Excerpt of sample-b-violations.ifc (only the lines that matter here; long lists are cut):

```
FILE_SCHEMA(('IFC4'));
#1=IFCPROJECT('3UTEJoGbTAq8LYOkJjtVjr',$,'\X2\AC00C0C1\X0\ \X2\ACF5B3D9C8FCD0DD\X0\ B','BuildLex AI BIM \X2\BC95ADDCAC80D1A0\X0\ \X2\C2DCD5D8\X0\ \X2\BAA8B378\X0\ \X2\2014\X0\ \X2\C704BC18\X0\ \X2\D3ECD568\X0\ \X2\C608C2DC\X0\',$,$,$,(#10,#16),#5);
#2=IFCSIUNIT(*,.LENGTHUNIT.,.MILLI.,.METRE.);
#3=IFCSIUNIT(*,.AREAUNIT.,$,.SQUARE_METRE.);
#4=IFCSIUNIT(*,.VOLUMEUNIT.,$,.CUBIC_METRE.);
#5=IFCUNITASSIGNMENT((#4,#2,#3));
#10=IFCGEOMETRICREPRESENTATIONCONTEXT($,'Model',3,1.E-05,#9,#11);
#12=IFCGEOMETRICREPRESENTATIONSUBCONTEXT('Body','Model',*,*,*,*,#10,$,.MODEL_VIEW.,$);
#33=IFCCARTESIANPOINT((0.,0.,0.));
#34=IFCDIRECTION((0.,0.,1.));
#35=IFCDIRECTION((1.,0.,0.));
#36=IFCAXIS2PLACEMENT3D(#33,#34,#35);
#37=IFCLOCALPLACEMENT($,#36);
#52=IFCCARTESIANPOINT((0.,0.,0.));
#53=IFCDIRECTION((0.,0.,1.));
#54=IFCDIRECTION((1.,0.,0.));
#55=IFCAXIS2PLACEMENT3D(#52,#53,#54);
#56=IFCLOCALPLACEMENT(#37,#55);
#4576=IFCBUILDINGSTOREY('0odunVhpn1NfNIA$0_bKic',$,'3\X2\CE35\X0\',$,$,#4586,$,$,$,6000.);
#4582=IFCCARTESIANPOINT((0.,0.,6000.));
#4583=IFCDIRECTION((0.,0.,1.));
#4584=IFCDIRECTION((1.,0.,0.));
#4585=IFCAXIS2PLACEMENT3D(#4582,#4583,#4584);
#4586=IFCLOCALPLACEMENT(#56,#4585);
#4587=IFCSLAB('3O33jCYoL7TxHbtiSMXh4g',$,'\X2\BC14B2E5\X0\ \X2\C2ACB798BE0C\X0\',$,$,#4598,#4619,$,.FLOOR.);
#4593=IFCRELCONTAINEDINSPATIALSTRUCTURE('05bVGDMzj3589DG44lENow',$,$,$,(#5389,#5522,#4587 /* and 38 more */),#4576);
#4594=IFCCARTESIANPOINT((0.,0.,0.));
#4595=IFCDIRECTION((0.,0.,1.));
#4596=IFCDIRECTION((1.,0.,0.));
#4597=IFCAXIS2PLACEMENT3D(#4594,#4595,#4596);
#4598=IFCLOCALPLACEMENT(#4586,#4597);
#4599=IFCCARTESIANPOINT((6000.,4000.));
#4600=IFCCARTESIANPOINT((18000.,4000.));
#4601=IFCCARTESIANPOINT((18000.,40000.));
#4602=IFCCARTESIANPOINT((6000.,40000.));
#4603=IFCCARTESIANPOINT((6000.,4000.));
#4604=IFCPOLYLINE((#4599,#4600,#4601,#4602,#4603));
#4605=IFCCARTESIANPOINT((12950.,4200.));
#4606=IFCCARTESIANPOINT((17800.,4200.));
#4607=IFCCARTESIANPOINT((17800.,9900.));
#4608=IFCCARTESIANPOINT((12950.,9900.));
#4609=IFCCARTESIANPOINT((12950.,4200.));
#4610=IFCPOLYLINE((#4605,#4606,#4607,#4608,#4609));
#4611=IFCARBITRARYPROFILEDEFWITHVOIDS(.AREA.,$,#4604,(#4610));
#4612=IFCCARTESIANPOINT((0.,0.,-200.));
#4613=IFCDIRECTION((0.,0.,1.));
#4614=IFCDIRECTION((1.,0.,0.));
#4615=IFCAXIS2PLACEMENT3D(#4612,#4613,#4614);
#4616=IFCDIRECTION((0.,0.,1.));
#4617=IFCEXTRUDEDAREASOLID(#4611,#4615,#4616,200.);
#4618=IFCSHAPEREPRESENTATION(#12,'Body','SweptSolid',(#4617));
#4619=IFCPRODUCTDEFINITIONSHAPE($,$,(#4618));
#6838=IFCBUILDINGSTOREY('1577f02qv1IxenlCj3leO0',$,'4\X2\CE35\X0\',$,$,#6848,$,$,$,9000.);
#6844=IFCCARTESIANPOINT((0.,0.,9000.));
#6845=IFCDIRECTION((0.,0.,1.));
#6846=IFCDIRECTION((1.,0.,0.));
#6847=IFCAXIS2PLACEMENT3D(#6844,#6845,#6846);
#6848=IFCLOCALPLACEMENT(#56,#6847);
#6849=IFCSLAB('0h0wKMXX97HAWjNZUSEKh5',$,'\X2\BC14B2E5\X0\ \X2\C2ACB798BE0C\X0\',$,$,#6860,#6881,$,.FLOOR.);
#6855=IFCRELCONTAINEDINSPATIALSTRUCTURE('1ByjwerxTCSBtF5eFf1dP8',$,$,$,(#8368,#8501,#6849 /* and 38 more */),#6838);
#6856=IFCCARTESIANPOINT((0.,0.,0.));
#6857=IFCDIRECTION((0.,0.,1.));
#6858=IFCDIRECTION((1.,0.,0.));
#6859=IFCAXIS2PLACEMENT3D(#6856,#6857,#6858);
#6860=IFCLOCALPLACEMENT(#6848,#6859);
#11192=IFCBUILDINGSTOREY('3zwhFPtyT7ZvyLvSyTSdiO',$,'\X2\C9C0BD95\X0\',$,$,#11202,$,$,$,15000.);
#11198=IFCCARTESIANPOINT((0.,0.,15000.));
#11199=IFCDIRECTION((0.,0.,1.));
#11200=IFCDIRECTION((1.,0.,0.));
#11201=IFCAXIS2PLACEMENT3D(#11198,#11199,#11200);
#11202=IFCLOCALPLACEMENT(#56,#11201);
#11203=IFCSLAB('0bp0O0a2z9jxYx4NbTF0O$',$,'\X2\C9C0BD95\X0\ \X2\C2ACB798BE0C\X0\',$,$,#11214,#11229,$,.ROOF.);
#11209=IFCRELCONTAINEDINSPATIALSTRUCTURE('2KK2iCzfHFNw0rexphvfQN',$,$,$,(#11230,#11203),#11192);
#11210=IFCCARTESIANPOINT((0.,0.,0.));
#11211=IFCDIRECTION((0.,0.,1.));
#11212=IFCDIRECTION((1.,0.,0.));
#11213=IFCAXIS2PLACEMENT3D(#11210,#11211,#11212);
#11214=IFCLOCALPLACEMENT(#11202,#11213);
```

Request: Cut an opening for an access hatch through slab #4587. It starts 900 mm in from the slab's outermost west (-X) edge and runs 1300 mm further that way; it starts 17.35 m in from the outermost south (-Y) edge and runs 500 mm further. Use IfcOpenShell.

```python
import numpy as np
import ifcopenshell
import ifcopenshell.api.feature
import ifcopenshell.api.geometry
import ifcopenshell.api.root
import ifcopenshell.geom
import ifcopenshell.util.placement
import ifcopenshell.util.representation
import ifcopenshell.util.shape
import ifcopenshell.util.unit

model = ifcopenshell.open("sample-b-violations.ifc")
unit_scale = ifcopenshell.util.unit.calculate_unit_scale(model)
settings = ifcopenshell.geom.settings()


def volume(element):
    """Net volume in cubic metres, openings subtracted."""
    shape = ifcopenshell.geom.create_shape(settings, element)
    return ifcopenshell.util.shape.get_volume(shape.geometry)


slab = model.by_id(4587)
before = volume(slab)

# Extent in the slab's own axes, in metres. The edges named are its -X and -Y sides.
slab_shape = ifcopenshell.geom.create_shape(settings, slab)
vertices = ifcopenshell.util.shape.get_vertices(slab_shape.geometry)
x_min, y_min, bottom = vertices.min(axis=0)
top = vertices[:, 2].max()

opening = ifcopenshell.api.root.create_entity(model, ifc_class="IfcOpeningElement", name="Access hatch opening", predefined_type="OPENING")
context = ifcopenshell.util.representation.get_context(model, "Model", "Body", "MODEL_VIEW")
width, depth = 1.3, 0.5
outline = [(0.0, 0.0), (width, 0.0), (width, depth), (0.0, depth), (0.0, 0.0)]
# Overshoot both faces by 50 mm so the cut is clean.
shape = ifcopenshell.api.geometry.add_slab_representation(
    model, context=context, depth=top - bottom + 0.1, polyline=outline
)
ifcopenshell.api.geometry.assign_representation(model, product=opening, representation=shape)

matrix = ifcopenshell.util.placement.get_local_placement(slab.ObjectPlacement)
matrix[:, 3] = matrix @ np.append(np.array([x_min + 0.9, y_min + 17.35, bottom - 0.05]) / unit_scale, 1.0)
ifcopenshell.api.geometry.edit_object_placement(model, product=opening, matrix=matrix, is_si=False)
ifcopenshell.api.feature.add_feature(model, feature=opening, element=slab)

after = volume(slab)

print(f"slab volume {before:.3f} -> {after:.3f} m3")

model.write("sample-b-violations_updated.ifc")
```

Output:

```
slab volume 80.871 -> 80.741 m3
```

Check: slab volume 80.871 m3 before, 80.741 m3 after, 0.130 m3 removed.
